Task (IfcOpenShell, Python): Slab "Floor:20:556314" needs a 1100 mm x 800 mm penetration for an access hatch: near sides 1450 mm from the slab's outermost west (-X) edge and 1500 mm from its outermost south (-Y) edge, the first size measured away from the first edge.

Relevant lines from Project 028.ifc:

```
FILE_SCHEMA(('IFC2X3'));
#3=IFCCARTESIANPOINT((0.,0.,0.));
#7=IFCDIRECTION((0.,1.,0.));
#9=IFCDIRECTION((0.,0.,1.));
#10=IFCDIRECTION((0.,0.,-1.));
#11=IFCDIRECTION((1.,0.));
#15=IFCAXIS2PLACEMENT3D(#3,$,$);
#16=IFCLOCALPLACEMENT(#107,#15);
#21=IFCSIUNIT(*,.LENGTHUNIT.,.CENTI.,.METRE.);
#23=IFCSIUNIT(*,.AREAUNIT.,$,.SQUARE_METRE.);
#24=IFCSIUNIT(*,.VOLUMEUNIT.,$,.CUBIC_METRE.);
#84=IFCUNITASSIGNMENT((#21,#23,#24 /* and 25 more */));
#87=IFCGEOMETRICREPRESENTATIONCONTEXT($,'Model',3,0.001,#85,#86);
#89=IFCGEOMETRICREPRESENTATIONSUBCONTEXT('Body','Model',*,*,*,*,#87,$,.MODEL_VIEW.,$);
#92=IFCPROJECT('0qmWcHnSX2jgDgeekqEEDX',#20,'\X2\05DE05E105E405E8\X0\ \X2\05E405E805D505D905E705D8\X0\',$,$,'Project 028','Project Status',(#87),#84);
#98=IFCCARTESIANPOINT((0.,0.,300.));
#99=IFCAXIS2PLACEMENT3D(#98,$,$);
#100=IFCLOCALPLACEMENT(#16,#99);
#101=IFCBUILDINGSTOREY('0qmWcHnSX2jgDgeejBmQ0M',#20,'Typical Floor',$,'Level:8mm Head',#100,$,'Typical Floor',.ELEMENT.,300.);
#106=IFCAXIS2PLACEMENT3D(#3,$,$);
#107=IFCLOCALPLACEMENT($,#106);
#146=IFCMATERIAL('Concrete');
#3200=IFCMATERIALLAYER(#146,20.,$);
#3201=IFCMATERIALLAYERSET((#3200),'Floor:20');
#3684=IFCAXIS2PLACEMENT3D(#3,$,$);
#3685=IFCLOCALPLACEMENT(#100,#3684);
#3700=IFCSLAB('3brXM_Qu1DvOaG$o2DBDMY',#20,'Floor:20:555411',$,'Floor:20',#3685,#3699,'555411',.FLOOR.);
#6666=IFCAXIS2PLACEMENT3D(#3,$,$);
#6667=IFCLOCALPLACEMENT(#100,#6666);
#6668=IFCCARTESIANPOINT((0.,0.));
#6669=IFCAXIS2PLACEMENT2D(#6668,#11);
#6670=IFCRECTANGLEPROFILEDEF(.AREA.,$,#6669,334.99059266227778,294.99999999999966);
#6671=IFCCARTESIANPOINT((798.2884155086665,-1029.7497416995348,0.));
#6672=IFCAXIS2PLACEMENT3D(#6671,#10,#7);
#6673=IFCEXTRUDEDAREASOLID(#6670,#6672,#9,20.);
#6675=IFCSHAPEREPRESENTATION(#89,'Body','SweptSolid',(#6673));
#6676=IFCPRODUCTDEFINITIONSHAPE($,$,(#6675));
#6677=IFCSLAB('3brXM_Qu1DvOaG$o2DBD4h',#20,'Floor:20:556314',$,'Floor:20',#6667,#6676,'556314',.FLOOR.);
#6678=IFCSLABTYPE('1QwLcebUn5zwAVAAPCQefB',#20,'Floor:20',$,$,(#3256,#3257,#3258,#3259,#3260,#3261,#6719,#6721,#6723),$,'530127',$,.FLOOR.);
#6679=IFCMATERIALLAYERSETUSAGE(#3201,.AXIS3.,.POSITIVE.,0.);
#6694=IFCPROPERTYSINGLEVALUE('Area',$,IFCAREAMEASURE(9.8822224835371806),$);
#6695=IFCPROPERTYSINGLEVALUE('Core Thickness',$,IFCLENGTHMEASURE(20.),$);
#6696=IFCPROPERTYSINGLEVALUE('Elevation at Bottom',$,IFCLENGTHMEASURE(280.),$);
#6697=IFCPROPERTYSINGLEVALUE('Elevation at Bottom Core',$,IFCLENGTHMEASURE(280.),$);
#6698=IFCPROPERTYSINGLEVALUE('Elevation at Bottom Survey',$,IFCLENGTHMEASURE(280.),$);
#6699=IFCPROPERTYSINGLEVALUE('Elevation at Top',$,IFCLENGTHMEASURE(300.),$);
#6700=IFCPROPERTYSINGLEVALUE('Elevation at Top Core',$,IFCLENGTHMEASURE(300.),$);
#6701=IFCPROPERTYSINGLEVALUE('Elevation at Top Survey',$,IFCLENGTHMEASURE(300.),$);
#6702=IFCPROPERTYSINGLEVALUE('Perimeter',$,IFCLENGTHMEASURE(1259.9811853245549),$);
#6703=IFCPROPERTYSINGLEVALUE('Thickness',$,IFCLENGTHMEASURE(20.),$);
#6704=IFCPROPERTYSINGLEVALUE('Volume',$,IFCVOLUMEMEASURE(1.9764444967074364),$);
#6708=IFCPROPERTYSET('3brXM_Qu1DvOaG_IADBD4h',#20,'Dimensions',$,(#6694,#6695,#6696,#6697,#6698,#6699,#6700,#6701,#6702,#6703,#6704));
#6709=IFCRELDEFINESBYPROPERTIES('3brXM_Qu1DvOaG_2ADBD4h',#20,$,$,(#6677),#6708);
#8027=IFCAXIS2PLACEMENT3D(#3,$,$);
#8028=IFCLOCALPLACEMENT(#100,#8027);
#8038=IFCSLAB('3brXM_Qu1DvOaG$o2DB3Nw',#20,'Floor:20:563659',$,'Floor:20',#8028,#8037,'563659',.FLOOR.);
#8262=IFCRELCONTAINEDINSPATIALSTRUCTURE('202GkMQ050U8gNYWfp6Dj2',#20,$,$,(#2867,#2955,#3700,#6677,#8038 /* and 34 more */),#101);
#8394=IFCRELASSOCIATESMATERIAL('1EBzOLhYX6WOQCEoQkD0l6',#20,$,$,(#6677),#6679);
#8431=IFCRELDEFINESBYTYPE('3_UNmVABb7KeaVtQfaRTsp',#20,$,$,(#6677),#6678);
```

```python
import numpy as np
import ifcopenshell
import ifcopenshell.api.feature
import ifcopenshell.api.geometry
import ifcopenshell.api.pset
import ifcopenshell.api.root
import ifcopenshell.geom
import ifcopenshell.util.element
import ifcopenshell.util.placement
import ifcopenshell.util.representation
import ifcopenshell.util.shape
import ifcopenshell.util.unit

model = ifcopenshell.open("Project 028.ifc")
unit_scale = ifcopenshell.util.unit.calculate_unit_scale(model)
area_scale = ifcopenshell.util.unit.calculate_unit_scale(model, "AREAUNIT")
volume_scale = ifcopenshell.util.unit.calculate_unit_scale(model, "VOLUMEUNIT")
settings = ifcopenshell.geom.settings()


def volume(element):
    """Net volume in cubic metres, openings subtracted."""
    shape = ifcopenshell.geom.create_shape(settings, element)
    return ifcopenshell.util.shape.get_volume(shape.geometry)


slab = model.by_guid("3brXM_Qu1DvOaG$o2DBD4h")
before = volume(slab)

# Extent in the slab's own axes, in metres. The edges named are its -X and -Y sides.
slab_shape = ifcopenshell.geom.create_shape(settings, slab)
vertices = ifcopenshell.util.shape.get_vertices(slab_shape.geometry)
x_min, y_min, bottom = vertices.min(axis=0)
top = vertices[:, 2].max()

opening = ifcopenshell.api.root.create_entity(model, ifc_class="IfcOpeningElement", name="Access hatch opening")
context = ifcopenshell.util.representation.get_context(model, "Model", "Body", "MODEL_VIEW")
width, depth = 1.1, 0.8
outline = [(0.0, 0.0), (width, 0.0), (width, depth), (0.0, depth), (0.0, 0.0)]
# Overshoot both faces by 50 mm so the cut is clean.
shape = ifcopenshell.api.geometry.add_slab_representation(
    model, context=context, depth=top - bottom + 0.1, polyline=outline
)
ifcopenshell.api.geometry.assign_representation(model, product=opening, representation=shape)

matrix = ifcopenshell.util.placement.get_local_placement(slab.ObjectPlacement)
matrix[:, 3] = matrix @ np.append(np.array([x_min + 1.45, y_min + 1.5, bottom - 0.05]) / unit_scale, 1.0)
ifcopenshell.api.geometry.edit_object_placement(model, product=opening, matrix=matrix, is_si=False)
ifcopenshell.api.feature.add_feature(model, feature=opening, element=slab)

after = volume(slab)

# Update the slab's stored quantities.
pset = model.by_id(ifcopenshell.util.element.get_pset(slab, "Dimensions", should_inherit=False)["id"])
ifcopenshell.api.pset.edit_pset(model, pset=pset, properties={
    "Area": model.create_entity("IfcAreaMeasure", after / (top - bottom) / area_scale),
    "Volume": model.create_entity("IfcVolumeMeasure", after / volume_scale),
})

print(f"slab volume {before:.3f} -> {after:.3f} m3")

model.write("Project 028_v2.ifc")
```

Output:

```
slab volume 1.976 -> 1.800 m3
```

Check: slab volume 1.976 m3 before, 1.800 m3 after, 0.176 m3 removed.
